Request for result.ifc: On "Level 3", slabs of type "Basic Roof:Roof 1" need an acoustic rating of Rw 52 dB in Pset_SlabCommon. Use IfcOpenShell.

First a look at what the model holds.

```python
import ifcopenshell
import ifcopenshell.util.element

model = ifcopenshell.open("result.ifc")
print(model.schema)
storey = next(s for s in model.by_type("IfcBuildingStorey") if s.Name == "Level 3")
slabs = [e for e in ifcopenshell.util.element.get_decomposition(storey) if e.is_a("IfcSlab")]
seen = {}
for e in slabs:
    element_type = ifcopenshell.util.element.get_type(e)
    key = (element_type.Name if element_type != e and element_type else None, ifcopenshell.util.element.get_pset(e, "Pset_SlabCommon", "AcousticRating"))
    seen[key] = seen.get(key, 0) + 1
for (name, value), count in sorted(seen.items(), key=str):
    print(count, "x", name, "|", value)
```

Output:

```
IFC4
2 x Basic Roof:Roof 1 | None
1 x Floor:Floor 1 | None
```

```python
import ifcopenshell
import ifcopenshell.api.pset
import ifcopenshell.util.element

model = ifcopenshell.open("result.ifc")

storey = next(s for s in model.by_type("IfcBuildingStorey") if s.Name == "Level 3")
slabs = [e for e in ifcopenshell.util.element.get_decomposition(storey) if e.is_a("IfcSlab")]

count = 0
for e in slabs:
    element_type = ifcopenshell.util.element.get_type(e)
    if element_type in (None, e) or element_type.Name != "Basic Roof:Roof 1":
        continue
    # add_pset returns the element's existing set when there is one.
    pset = ifcopenshell.api.pset.add_pset(model, product=e, name="Pset_SlabCommon")
    ifcopenshell.api.pset.edit_pset(model, pset=pset, properties={"AcousticRating": "Rw 52 dB"})
    count += 1

print(count, "slabs updated")

model.write("result_v2.ifc")
```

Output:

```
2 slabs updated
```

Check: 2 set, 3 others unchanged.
